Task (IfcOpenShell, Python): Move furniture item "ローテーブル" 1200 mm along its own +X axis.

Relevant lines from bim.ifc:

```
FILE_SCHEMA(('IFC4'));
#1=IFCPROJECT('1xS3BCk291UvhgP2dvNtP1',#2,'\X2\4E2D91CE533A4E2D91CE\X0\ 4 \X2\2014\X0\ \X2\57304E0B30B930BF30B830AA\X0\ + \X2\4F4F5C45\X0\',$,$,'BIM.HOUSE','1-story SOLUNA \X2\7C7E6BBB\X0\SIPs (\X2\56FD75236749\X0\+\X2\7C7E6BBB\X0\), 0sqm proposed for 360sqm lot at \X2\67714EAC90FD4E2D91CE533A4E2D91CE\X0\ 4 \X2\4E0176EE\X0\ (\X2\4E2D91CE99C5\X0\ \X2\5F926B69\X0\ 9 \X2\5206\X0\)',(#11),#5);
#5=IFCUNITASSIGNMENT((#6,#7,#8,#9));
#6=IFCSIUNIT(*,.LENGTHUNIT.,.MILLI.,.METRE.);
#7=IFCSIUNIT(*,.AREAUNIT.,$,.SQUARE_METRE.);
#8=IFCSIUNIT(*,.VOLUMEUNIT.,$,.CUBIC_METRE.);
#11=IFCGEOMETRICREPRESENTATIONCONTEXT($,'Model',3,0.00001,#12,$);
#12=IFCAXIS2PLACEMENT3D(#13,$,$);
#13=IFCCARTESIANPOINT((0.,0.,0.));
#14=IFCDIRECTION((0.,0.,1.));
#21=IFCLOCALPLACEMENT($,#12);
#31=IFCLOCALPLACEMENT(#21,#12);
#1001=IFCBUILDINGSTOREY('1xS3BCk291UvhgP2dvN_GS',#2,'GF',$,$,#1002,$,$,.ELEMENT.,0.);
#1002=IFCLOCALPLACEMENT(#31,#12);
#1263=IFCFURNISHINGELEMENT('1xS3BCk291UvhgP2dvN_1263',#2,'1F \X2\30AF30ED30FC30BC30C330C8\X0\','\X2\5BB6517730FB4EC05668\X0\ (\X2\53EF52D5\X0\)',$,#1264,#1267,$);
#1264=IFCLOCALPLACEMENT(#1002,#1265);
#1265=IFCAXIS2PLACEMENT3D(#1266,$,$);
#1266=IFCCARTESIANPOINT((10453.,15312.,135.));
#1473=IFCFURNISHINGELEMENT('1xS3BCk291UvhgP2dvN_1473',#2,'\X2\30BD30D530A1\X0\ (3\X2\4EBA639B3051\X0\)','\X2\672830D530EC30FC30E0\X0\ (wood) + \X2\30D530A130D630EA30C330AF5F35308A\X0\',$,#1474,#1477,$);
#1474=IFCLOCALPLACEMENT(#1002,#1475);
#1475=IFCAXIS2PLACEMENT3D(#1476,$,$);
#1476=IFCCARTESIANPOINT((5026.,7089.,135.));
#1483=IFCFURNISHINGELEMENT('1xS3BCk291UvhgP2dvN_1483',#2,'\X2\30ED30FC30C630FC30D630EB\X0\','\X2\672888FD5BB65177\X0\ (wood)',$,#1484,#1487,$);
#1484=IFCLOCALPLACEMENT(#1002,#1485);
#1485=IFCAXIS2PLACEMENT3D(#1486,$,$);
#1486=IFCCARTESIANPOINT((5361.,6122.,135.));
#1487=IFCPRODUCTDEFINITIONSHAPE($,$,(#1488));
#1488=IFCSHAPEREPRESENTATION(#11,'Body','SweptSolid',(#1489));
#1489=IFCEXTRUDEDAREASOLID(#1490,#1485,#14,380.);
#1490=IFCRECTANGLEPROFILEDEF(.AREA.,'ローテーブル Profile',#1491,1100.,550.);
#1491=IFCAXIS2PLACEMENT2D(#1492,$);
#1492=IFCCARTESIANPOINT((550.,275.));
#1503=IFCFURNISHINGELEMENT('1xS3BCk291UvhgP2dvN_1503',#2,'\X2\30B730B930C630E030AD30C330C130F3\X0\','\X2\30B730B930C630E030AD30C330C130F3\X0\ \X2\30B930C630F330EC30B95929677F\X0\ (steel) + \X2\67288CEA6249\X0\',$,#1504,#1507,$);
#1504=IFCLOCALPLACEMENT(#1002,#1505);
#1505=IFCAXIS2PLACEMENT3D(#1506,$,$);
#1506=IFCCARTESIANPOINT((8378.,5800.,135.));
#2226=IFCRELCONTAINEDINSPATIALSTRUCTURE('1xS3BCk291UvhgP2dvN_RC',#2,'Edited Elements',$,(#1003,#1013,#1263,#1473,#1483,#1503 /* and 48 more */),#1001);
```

```python
import ifcopenshell
import ifcopenshell.api.geometry
import ifcopenshell.util.placement

model = ifcopenshell.open("bim.ifc")

item = model.by_guid("1xS3BCk291UvhgP2dvN_1483")
matrix = ifcopenshell.util.placement.get_local_placement(item.ObjectPlacement)
matrix[:3, 3] += matrix[:3, 0] * 1200.0
ifcopenshell.api.geometry.edit_object_placement(model, product=item, matrix=matrix, is_si=False)

print(ifcopenshell.util.placement.get_local_placement(item.ObjectPlacement).round(3) + 0.0)

model.write("bim-out.ifc")
```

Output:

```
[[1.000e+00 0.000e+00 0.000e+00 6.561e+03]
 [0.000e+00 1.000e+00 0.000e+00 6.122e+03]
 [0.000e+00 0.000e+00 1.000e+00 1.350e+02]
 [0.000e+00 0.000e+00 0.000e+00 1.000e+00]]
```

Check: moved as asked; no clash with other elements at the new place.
